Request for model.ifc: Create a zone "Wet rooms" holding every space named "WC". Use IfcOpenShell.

First a look at what the model holds.

```python
import ifcopenshell

model = ifcopenshell.open("model.ifc")
print(model.schema)
seen = {}
for space in model.by_type("IfcSpace"):
    seen[space.LongName] = seen.get(space.LongName, 0) + 1
for name, count in sorted(seen.items(), key=str):
    print(count, "x", name)
print("zones:", [z.Name for z in model.by_type("IfcZone")][:20])
```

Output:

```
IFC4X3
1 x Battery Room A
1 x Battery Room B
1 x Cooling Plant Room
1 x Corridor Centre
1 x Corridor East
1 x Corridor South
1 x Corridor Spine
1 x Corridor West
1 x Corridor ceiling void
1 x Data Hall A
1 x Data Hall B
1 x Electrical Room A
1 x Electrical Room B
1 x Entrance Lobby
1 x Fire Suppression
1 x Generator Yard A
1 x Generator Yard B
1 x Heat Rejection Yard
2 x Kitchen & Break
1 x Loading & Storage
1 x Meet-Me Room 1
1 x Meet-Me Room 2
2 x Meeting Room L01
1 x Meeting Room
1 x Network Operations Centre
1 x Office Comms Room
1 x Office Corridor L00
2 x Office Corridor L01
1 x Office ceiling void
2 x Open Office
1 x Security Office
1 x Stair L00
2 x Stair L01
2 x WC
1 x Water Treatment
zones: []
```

```python
import ifcopenshell
import ifcopenshell.api.group
import ifcopenshell.api.root

model = ifcopenshell.open("model.ifc")

names = {"WC"}
spaces = [s for s in model.by_type("IfcSpace") if s.LongName in names]

zone = ifcopenshell.api.root.create_entity(model, ifc_class="IfcZone", name="Wet rooms")
ifcopenshell.api.group.assign_group(model, products=spaces, group=zone)
print(len(spaces), "spaces in", zone.Name)

model.write("model_updated.ifc")
```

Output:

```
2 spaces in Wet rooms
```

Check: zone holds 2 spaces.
